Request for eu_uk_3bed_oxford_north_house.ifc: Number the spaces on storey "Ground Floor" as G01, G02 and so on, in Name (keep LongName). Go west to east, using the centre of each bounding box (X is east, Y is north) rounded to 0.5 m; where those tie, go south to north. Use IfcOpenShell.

First a look at what the model holds.

```python
import ifcopenshell
import ifcopenshell.util.element
import ifcopenshell.util.placement

model = ifcopenshell.open("eu_uk_3bed_oxford_north_house.ifc")
print(model.schema)
storey = next(s for s in model.by_type("IfcBuildingStorey") if s.Name == "Ground Floor")
spaces = [e for e in ifcopenshell.util.element.get_decomposition(storey) if e.is_a("IfcSpace")]
for e in sorted(spaces, key=lambda e: e.id()):
    origin = ifcopenshell.util.placement.get_local_placement(e.ObjectPlacement)[:3, 3]
    print(e.id(), e.Name, e.LongName, origin.round(2) + 0.0, sep=" | ")
```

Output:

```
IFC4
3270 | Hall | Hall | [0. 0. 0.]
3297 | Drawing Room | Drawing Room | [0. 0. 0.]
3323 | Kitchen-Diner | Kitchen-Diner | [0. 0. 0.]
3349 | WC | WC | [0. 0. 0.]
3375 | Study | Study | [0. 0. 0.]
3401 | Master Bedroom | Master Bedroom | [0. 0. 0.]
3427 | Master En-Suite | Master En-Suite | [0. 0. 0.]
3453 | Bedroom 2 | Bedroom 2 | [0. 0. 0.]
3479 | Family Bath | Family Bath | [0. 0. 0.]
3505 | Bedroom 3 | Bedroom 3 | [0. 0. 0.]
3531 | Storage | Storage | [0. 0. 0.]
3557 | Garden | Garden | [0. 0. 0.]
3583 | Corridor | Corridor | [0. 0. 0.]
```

```python
import ifcopenshell
import ifcopenshell.geom
import ifcopenshell.util.element
import ifcopenshell.util.shape

model = ifcopenshell.open("eu_uk_3bed_oxford_north_house.ifc")
settings = ifcopenshell.geom.settings()
settings.set("use-world-coords", True)


def centre(element):
    shape = ifcopenshell.geom.create_shape(settings, element)
    return ifcopenshell.util.shape.get_bbox_centroid(shape.geometry)


storey = next(s for s in model.by_type("IfcBuildingStorey") if s.Name == "Ground Floor")
spaces = [e for e in ifcopenshell.util.element.get_decomposition(storey) if e.is_a("IfcSpace")]

# Insertion points can sit at a corner or the storey origin, so sort by the geometry (in metres).
centres = {e: centre(e) for e in spaces}
spaces.sort(key=lambda e: (round(centres[e][0] / 0.5), centres[e][1]))

for i, e in enumerate(spaces, start=1):
    number = f"G{i:02d}"
    e.Name = number
    print(e.id(), number)

model.write("eu_uk_3bed_oxford_north_house-out.ifc")
```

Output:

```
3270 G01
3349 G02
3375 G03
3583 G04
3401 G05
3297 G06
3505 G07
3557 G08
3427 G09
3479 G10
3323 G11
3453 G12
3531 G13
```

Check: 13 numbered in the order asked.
